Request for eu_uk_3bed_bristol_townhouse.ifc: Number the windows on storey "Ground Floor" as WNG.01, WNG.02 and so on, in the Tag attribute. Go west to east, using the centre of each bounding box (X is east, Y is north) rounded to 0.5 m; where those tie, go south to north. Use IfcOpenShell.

First a look at what the model holds.

```python
import ifcopenshell
import ifcopenshell.util.element
import ifcopenshell.util.placement

model = ifcopenshell.open("eu_uk_3bed_bristol_townhouse.ifc")
print(model.schema)
storey = next(s for s in model.by_type("IfcBuildingStorey") if s.Name == "Ground Floor")
windows = [e for e in ifcopenshell.util.element.get_decomposition(storey) if e.is_a("IfcWindow")]
for e in sorted(windows, key=lambda e: e.id()):
    origin = ifcopenshell.util.placement.get_local_placement(e.ObjectPlacement)[:3, 3]
    print(e.id(), e.Tag, e.Name, origin.round(2) + 0.0, sep=" | ")
```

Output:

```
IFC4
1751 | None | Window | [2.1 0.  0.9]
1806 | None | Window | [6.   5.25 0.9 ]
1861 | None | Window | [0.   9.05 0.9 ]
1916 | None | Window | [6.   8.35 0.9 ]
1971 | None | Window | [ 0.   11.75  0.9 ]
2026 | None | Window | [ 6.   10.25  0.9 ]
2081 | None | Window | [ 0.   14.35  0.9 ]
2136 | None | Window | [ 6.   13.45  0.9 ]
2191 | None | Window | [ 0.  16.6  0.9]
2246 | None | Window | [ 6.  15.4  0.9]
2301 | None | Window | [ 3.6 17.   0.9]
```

```python
import ifcopenshell
import ifcopenshell.geom
import ifcopenshell.util.element
import ifcopenshell.util.shape

model = ifcopenshell.open("eu_uk_3bed_bristol_townhouse.ifc")
settings = ifcopenshell.geom.settings()
settings.set("use-world-coords", True)


def centre(element):
    shape = ifcopenshell.geom.create_shape(settings, element)
    return ifcopenshell.util.shape.get_bbox_centroid(shape.geometry)


storey = next(s for s in model.by_type("IfcBuildingStorey") if s.Name == "Ground Floor")
windows = [e for e in ifcopenshell.util.element.get_decomposition(storey) if e.is_a("IfcWindow")]

# Insertion points can sit at a corner or the storey origin, so sort by the geometry (in metres).
centres = {e: centre(e) for e in windows}
windows.sort(key=lambda e: (round(centres[e][0] / 0.5), centres[e][1]))

for i, e in enumerate(windows, start=1):
    number = f"WNG.{i:02d}"
    e.Tag = number
    print(e.id(), number)

model.write("eu_uk_3bed_bristol_townhouse_updated.ifc")
```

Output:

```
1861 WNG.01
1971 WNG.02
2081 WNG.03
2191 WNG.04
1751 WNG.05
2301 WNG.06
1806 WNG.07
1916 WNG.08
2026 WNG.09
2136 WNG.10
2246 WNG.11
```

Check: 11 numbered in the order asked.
